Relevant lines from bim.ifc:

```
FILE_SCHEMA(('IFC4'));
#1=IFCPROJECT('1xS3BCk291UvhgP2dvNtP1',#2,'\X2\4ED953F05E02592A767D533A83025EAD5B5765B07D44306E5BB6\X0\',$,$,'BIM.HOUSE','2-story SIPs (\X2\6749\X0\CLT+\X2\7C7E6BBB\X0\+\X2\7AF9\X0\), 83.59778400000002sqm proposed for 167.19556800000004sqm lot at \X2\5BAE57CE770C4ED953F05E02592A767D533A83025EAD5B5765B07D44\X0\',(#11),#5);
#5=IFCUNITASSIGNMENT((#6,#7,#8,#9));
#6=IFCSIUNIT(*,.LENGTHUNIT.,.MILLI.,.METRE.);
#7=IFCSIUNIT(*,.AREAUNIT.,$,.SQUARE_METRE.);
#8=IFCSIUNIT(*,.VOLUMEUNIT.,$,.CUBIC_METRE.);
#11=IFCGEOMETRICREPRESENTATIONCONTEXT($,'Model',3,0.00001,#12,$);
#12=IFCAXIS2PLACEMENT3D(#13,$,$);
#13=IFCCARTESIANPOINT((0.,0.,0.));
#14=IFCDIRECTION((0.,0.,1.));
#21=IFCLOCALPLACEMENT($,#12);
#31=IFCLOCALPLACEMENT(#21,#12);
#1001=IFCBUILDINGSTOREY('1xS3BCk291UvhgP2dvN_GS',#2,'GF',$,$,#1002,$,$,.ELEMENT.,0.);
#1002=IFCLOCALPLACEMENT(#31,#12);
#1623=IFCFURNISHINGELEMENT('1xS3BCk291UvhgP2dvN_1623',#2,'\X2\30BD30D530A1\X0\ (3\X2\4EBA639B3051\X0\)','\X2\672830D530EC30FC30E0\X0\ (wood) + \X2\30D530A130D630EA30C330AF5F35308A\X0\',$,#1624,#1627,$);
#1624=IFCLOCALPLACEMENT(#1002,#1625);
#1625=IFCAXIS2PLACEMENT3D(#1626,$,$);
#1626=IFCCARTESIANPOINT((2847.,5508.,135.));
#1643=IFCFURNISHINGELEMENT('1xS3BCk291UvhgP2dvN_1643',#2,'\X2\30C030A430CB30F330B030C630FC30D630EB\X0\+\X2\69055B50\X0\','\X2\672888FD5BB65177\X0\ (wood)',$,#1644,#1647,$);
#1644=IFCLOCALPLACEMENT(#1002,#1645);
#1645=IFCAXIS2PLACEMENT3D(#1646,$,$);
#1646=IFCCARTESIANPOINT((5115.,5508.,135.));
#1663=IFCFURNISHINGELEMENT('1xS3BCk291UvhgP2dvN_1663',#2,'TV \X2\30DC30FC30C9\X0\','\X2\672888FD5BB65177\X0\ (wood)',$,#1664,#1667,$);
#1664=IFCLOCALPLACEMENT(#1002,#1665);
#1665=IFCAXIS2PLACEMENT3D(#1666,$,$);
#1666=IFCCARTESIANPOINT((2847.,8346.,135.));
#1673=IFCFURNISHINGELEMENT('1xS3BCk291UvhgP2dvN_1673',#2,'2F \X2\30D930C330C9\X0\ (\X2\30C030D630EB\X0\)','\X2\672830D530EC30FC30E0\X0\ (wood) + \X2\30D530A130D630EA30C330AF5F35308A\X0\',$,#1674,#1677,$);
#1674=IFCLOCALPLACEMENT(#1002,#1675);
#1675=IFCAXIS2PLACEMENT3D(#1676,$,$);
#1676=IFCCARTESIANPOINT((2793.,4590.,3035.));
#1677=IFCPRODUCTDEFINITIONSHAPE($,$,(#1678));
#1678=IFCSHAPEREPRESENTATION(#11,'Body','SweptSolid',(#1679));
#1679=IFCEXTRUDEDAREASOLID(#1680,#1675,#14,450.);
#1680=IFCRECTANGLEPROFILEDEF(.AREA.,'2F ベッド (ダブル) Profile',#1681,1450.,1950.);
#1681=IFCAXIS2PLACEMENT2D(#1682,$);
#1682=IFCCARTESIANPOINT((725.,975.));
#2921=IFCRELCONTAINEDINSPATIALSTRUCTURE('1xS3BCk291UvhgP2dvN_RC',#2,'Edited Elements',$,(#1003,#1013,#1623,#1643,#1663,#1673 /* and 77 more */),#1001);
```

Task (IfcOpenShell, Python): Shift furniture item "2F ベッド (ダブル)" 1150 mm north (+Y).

```python
import ifcopenshell
import ifcopenshell.api.geometry
import ifcopenshell.util.placement
import ifcopenshell.util.unit

model = ifcopenshell.open("bim.ifc")
unit_scale = ifcopenshell.util.unit.calculate_unit_scale(model)

item = model.by_guid("1xS3BCk291UvhgP2dvN_1673")
matrix = ifcopenshell.util.placement.get_local_placement(item.ObjectPlacement)
matrix[1, 3] += 1.15 / unit_scale
ifcopenshell.api.geometry.edit_object_placement(model, product=item, matrix=matrix, is_si=False)

print(ifcopenshell.util.placement.get_local_placement(item.ObjectPlacement).round(3) + 0.0)

model.write("bim_rev.ifc")
```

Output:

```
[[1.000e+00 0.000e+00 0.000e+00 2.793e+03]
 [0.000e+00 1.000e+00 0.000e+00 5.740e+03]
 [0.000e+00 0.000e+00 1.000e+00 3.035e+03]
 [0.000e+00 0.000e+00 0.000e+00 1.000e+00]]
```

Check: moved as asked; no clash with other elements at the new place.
